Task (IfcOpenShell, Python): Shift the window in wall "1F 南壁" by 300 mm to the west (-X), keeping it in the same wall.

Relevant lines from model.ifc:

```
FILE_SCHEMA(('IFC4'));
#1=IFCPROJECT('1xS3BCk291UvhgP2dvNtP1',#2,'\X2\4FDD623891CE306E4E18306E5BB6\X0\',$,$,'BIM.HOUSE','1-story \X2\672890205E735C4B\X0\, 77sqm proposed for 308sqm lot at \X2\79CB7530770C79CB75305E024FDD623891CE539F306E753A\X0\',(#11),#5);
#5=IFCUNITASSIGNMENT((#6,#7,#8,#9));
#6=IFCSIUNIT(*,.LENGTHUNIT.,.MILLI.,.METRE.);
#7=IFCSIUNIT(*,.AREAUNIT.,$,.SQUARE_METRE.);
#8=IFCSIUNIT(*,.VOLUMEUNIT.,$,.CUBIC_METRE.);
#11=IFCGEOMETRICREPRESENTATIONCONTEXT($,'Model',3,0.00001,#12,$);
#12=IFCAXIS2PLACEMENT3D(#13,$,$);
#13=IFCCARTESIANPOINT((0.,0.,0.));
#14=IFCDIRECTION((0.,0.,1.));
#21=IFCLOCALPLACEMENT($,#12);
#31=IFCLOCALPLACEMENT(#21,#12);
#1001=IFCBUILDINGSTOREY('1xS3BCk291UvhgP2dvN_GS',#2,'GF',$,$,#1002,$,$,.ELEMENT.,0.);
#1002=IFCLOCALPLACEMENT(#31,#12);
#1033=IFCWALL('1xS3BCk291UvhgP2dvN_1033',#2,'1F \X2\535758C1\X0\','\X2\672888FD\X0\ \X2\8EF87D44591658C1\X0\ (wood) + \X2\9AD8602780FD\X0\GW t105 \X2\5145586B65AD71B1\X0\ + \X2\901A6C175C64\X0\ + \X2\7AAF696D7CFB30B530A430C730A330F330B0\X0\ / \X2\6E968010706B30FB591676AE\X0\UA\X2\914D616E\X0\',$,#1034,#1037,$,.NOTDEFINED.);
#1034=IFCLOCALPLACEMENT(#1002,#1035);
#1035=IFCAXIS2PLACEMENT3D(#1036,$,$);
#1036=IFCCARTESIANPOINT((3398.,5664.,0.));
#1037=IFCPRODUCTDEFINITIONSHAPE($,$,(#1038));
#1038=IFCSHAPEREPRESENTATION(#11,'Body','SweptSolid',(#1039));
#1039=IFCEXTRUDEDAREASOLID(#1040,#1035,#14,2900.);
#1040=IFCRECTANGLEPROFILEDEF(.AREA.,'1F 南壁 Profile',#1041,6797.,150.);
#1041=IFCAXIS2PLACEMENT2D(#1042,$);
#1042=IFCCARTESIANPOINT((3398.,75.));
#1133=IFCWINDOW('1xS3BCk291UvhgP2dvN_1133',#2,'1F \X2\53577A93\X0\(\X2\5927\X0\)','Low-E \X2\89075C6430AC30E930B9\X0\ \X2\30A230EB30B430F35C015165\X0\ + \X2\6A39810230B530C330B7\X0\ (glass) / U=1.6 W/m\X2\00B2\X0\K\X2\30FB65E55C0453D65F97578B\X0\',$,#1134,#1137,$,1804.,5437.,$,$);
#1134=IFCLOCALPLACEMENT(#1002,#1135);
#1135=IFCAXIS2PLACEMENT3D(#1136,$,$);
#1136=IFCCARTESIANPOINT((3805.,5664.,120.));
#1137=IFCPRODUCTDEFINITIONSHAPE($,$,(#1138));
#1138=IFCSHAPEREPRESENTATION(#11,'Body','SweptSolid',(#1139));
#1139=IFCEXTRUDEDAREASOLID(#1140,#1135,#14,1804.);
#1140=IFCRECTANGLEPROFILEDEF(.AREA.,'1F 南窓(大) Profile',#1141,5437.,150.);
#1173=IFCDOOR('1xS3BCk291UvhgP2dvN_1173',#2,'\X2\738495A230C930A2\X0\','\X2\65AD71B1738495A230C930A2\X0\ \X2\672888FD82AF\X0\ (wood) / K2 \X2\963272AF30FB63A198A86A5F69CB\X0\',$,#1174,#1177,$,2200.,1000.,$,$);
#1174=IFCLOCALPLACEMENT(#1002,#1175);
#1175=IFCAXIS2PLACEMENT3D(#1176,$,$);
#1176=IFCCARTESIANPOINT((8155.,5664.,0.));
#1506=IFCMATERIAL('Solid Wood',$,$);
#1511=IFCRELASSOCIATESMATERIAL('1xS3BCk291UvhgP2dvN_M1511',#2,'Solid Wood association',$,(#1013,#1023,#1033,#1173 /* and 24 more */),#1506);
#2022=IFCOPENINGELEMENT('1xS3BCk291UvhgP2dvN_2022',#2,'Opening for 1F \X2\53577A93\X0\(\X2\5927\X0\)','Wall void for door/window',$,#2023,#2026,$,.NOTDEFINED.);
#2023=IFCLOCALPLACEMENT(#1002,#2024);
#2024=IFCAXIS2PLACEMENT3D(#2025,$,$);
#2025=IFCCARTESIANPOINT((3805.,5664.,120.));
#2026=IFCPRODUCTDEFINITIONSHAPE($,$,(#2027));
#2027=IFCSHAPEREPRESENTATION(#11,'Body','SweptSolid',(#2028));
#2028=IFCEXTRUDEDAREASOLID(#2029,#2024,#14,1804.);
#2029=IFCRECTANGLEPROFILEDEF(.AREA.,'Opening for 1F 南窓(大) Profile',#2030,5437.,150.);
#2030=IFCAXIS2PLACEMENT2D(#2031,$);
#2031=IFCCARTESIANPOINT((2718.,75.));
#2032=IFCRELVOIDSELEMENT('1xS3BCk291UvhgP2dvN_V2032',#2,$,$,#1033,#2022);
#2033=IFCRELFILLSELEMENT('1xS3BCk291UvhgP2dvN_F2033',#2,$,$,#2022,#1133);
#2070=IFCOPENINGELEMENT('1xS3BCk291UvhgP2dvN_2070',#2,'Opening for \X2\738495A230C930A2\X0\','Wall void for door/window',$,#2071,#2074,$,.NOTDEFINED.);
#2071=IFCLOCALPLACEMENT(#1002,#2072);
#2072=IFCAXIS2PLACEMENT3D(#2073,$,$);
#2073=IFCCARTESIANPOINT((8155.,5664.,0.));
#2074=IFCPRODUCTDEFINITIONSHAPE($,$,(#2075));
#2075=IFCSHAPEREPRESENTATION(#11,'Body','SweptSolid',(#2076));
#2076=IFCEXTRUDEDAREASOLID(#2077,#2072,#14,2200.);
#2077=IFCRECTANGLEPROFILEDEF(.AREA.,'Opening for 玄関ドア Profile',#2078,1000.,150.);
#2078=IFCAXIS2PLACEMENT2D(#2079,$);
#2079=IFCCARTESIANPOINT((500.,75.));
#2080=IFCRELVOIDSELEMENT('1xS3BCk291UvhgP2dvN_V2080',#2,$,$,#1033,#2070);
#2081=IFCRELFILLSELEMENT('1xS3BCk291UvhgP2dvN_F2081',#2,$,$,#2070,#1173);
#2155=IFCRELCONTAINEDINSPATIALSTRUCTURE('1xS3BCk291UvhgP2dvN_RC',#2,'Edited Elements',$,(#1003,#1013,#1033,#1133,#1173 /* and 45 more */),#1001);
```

```python
import ifcopenshell
import ifcopenshell.api.geometry
import ifcopenshell.util.placement
import ifcopenshell.util.unit

model = ifcopenshell.open("model.ifc")
unit_scale = ifcopenshell.util.unit.calculate_unit_scale(model)

window = model.by_guid("1xS3BCk291UvhgP2dvN_1133")
opening = window.FillsVoids[0].RelatingOpeningElement
wall = opening.VoidsElements[0].RelatingBuildingElement

wall_matrix = ifcopenshell.util.placement.get_local_placement(wall.ObjectPlacement)
shift = wall_matrix[:3, 0] * -0.3 / unit_scale
before = ifcopenshell.util.placement.get_local_placement(window.ObjectPlacement)[:3, 3].copy()

# The window is not placed relative to its opening, so move both.
for product in (opening, window):
    matrix = ifcopenshell.util.placement.get_local_placement(product.ObjectPlacement)
    matrix[:3, 3] += shift
    ifcopenshell.api.geometry.edit_object_placement(model, product=product, matrix=matrix, is_si=False)

after = ifcopenshell.util.placement.get_local_placement(window.ObjectPlacement)[:3, 3]
print("window moved by", (after - before).round(3) + 0.0)

model.write("model_v2.ifc")
```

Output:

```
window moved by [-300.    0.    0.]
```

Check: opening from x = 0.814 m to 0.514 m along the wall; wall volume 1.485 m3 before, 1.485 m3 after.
